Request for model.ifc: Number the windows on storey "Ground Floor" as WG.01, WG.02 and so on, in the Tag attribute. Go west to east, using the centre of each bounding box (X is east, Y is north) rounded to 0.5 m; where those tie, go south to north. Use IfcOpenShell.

First a look at what the model holds.

```python
import ifcopenshell
import ifcopenshell.util.element
import ifcopenshell.util.placement

model = ifcopenshell.open("model.ifc")
print(model.schema)
storey = next(s for s in model.by_type("IfcBuildingStorey") if s.Name == "Ground Floor")
windows = [e for e in ifcopenshell.util.element.get_decomposition(storey) if e.is_a("IfcWindow")]
for e in sorted(windows, key=lambda e: e.id()):
    origin = ifcopenshell.util.placement.get_local_placement(e.ObjectPlacement)[:3, 3]
    print(e.id(), e.Tag, e.Name, origin.round(2) + 0.0, sep=" | ")
```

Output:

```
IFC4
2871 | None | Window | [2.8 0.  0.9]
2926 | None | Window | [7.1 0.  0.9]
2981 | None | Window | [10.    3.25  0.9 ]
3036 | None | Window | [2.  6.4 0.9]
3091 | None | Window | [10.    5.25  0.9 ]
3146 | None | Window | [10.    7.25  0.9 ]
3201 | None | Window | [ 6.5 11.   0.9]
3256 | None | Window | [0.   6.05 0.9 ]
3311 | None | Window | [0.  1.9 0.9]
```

```python
import ifcopenshell
import ifcopenshell.geom
import ifcopenshell.util.element
import ifcopenshell.util.shape

model = ifcopenshell.open("model.ifc")
settings = ifcopenshell.geom.settings()
settings.set("use-world-coords", True)


def centre(element):
    shape = ifcopenshell.geom.create_shape(settings, element)
    return ifcopenshell.util.shape.get_bbox_centroid(shape.geometry)


storey = next(s for s in model.by_type("IfcBuildingStorey") if s.Name == "Ground Floor")
windows = [e for e in ifcopenshell.util.element.get_decomposition(storey) if e.is_a("IfcWindow")]

# Insertion points can sit at a corner or the storey origin, so sort by the geometry (in metres).
centres = {e: centre(e) for e in windows}
windows.sort(key=lambda e: (round(centres[e][0] / 0.5), centres[e][1]))

for i, e in enumerate(windows, start=1):
    number = f"WG.{i:02d}"
    e.Tag = number
    print(e.id(), number)

model.write("model_updated.ifc")
```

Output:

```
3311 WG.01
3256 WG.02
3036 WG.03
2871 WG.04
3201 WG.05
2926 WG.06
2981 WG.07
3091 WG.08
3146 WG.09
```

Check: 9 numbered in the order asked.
